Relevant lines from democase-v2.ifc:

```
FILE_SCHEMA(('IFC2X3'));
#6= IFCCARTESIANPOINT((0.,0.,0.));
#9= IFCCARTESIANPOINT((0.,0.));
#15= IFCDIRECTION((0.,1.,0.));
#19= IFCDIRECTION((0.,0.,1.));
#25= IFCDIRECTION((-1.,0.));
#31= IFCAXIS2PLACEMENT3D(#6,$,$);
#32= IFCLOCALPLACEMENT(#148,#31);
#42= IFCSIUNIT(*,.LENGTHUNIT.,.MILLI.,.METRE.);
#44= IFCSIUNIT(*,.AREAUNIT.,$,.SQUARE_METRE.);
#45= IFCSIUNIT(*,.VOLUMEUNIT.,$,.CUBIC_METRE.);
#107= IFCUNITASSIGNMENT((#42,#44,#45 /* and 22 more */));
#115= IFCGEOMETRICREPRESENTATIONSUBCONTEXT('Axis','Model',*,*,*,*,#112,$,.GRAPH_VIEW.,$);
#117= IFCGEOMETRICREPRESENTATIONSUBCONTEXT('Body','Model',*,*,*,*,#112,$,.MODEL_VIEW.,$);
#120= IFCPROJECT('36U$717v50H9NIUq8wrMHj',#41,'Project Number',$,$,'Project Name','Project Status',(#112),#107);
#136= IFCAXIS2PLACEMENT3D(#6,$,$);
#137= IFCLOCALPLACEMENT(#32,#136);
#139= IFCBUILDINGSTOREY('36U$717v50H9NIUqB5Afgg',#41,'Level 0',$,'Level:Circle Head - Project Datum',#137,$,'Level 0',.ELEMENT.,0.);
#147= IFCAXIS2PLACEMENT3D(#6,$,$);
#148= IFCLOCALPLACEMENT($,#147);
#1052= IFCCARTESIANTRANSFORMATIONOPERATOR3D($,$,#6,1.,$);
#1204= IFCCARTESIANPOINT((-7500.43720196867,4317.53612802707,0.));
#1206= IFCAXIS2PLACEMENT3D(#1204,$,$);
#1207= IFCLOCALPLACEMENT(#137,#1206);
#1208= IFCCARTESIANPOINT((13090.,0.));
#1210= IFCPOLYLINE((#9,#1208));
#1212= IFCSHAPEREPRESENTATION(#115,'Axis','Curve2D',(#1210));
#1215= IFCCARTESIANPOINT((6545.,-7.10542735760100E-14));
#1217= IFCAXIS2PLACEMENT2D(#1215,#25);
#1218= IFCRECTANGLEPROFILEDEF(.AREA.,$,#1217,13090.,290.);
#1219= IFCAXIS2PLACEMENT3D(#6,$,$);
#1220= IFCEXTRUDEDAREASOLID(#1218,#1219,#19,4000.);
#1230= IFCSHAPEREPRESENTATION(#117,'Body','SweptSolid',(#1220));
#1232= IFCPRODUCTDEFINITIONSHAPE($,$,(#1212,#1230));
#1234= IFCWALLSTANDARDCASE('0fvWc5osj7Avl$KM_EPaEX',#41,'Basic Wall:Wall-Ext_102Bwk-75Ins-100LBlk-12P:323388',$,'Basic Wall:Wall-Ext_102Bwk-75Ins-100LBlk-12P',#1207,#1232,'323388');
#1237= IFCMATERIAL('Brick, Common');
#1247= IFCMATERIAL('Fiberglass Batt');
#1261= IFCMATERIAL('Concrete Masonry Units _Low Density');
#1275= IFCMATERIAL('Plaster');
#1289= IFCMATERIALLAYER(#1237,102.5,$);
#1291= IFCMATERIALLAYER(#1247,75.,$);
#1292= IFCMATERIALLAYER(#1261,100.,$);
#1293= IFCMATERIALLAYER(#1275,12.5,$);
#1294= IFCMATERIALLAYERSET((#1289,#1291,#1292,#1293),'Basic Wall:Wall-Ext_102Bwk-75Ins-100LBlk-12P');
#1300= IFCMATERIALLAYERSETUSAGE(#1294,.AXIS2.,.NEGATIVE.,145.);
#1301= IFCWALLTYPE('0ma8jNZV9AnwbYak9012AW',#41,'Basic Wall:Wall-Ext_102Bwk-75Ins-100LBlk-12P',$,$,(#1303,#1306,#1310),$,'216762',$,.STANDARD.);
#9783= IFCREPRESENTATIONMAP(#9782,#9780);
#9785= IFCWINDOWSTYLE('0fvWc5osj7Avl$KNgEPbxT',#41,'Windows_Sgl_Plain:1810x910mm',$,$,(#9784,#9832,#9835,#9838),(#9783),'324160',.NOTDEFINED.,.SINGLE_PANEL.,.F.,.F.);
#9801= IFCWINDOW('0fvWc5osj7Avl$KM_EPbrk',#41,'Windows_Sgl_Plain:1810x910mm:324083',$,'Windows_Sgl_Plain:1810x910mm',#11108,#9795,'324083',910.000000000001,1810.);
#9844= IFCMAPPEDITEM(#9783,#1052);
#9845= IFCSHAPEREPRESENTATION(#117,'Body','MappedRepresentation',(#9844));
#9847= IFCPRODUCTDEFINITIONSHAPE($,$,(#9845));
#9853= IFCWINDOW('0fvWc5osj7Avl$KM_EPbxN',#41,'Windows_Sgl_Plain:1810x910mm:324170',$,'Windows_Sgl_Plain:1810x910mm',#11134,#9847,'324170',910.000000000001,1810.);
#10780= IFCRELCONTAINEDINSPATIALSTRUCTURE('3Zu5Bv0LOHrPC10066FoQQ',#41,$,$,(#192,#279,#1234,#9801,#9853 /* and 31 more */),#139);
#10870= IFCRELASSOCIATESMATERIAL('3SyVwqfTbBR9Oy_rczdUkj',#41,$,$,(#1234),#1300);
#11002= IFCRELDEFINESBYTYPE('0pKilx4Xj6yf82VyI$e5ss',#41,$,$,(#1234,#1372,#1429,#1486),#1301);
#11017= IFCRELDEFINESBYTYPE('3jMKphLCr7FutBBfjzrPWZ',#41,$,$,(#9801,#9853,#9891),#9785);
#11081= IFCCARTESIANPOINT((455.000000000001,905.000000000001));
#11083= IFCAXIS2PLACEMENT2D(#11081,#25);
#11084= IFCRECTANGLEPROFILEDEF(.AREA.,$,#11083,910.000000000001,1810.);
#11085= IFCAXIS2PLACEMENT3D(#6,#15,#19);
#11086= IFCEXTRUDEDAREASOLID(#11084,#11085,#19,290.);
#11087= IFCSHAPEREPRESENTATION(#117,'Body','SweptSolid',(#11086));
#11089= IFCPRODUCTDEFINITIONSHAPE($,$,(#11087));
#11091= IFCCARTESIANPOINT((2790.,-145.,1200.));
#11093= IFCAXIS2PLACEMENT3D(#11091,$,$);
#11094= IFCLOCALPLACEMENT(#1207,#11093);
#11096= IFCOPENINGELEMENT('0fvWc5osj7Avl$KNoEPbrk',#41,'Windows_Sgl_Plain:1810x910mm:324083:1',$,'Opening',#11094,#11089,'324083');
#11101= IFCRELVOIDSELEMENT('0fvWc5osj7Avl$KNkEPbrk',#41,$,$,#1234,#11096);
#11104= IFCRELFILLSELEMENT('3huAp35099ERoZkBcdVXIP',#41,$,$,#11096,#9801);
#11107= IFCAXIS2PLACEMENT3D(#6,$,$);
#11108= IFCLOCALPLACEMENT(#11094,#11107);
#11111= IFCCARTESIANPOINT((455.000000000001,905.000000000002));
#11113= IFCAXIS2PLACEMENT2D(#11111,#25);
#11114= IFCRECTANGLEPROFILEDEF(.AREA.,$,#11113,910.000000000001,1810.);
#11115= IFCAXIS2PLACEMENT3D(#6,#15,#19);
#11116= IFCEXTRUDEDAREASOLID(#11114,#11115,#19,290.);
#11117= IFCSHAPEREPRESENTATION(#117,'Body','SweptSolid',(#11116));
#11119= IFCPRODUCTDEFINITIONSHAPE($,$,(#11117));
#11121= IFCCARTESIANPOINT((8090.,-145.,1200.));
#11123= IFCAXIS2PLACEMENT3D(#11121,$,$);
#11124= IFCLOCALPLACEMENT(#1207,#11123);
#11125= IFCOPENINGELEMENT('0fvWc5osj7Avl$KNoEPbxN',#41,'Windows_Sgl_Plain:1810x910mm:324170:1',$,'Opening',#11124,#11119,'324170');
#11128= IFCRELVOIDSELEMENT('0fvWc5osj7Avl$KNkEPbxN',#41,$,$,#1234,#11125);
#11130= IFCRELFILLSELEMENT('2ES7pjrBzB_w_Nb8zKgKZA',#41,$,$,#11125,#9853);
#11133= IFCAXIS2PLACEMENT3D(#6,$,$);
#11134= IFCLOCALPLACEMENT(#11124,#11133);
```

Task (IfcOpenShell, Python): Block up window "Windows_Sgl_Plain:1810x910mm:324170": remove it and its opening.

```python
import ifcopenshell
import ifcopenshell.api.feature
import ifcopenshell.api.root
import ifcopenshell.geom
import ifcopenshell.util.shape

model = ifcopenshell.open("democase-v2.ifc")
settings = ifcopenshell.geom.settings()


def volume(element):
    """Net volume in cubic metres, openings subtracted."""
    shape = ifcopenshell.geom.create_shape(settings, element)
    return ifcopenshell.util.shape.get_volume(shape.geometry)


window = model.by_guid("0fvWc5osj7Avl$KM_EPbxN")
opening = window.FillsVoids[0].RelatingOpeningElement
wall = opening.VoidsElements[0].RelatingBuildingElement
before = volume(wall)

ifcopenshell.api.root.remove_product(model, product=window)
ifcopenshell.api.feature.remove_feature(model, feature=opening)

after = volume(wall)

print(f"wall volume {before:.3f} -> {after:.3f} m3")

model.write("democase-v2-out.ifc")
```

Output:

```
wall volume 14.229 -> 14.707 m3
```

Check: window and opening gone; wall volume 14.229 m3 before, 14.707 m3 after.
